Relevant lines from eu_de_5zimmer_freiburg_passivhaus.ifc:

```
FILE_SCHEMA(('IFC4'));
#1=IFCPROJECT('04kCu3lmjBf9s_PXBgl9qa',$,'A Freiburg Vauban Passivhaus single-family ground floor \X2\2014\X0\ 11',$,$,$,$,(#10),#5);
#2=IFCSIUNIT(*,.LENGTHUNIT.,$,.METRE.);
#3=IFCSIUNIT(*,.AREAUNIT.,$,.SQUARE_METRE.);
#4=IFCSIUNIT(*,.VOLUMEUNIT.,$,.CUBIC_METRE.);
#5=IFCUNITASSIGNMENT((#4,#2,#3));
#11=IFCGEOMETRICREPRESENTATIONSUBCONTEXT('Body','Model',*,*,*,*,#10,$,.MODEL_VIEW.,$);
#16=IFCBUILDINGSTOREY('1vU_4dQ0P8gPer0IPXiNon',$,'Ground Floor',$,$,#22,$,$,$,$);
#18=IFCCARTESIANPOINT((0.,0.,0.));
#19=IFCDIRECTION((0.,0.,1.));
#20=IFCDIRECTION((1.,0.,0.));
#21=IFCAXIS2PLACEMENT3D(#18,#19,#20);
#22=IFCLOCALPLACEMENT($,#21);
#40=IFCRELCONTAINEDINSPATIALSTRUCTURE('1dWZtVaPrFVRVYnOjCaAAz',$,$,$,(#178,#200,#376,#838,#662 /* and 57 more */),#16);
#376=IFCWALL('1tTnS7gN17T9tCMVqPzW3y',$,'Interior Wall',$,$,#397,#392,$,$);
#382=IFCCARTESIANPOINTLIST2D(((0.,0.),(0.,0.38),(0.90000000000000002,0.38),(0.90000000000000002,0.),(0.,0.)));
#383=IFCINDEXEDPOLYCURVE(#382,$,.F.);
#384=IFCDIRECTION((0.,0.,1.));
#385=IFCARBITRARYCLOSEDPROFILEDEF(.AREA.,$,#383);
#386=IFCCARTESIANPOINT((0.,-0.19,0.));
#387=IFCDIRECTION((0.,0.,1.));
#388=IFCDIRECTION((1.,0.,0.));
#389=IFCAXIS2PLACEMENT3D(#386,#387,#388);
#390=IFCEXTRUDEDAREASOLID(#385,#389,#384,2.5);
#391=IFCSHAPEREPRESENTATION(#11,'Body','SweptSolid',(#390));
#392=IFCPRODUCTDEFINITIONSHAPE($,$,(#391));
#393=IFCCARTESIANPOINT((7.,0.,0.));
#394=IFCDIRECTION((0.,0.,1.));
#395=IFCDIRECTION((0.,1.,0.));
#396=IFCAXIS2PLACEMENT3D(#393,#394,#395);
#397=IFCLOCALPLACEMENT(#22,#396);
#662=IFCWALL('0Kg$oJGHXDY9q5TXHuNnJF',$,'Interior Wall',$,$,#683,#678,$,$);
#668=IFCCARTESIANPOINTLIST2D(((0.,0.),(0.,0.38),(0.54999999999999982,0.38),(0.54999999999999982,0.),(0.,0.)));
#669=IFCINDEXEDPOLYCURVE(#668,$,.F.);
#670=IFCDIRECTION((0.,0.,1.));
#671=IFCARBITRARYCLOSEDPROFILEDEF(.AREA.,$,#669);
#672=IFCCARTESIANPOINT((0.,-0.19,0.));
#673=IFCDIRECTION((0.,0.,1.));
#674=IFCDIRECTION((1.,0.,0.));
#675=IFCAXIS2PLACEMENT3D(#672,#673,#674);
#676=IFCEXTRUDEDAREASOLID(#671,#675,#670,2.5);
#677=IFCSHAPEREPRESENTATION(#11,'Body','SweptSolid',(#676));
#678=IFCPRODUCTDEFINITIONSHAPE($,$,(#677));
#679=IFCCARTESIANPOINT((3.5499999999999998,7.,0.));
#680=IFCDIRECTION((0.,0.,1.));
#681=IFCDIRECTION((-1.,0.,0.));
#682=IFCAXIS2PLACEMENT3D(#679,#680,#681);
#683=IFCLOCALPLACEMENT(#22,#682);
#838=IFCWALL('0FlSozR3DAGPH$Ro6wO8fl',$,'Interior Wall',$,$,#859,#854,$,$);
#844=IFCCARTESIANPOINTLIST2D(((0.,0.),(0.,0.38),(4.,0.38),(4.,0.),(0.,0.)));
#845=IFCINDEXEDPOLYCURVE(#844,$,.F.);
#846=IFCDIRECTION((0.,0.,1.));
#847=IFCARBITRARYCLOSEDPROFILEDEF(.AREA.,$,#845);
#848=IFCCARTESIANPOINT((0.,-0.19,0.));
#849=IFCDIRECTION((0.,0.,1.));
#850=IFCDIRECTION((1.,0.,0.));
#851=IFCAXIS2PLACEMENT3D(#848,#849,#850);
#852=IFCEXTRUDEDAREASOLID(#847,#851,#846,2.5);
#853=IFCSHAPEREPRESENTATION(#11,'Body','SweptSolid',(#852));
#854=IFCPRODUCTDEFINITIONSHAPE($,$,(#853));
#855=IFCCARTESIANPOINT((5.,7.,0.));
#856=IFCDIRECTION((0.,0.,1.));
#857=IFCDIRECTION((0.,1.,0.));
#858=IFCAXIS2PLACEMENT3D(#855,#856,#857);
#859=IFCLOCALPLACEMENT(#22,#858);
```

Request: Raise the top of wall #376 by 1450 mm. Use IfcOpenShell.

```python
import ifcopenshell
import ifcopenshell.geom
import ifcopenshell.util.representation
import ifcopenshell.util.shape
import ifcopenshell.util.unit

model = ifcopenshell.open("eu_de_5zimmer_freiburg_passivhaus.ifc")
unit_scale = ifcopenshell.util.unit.calculate_unit_scale(model)
settings = ifcopenshell.geom.settings()


def volume(element):
    """Net volume in cubic metres, openings subtracted."""
    shape = ifcopenshell.geom.create_shape(settings, element)
    return ifcopenshell.util.shape.get_volume(shape.geometry)


wall = model.by_guid("1tTnS7gN17T9tCMVqPzW3y")
before = volume(wall)

body = ifcopenshell.util.representation.get_representation(wall, "Model", "Body")
solid = body.Items[0]
old_height = solid.Depth
solid.Depth += 1.45 / unit_scale
after = volume(wall)

print(f"height {old_height:g} -> {solid.Depth:g}, volume {before:.3f} -> {after:.3f} m3")

model.write("eu_de_5zimmer_freiburg_passivhaus-out.ifc")
```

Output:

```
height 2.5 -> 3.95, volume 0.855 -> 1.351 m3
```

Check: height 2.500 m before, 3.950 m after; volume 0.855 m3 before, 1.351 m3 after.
